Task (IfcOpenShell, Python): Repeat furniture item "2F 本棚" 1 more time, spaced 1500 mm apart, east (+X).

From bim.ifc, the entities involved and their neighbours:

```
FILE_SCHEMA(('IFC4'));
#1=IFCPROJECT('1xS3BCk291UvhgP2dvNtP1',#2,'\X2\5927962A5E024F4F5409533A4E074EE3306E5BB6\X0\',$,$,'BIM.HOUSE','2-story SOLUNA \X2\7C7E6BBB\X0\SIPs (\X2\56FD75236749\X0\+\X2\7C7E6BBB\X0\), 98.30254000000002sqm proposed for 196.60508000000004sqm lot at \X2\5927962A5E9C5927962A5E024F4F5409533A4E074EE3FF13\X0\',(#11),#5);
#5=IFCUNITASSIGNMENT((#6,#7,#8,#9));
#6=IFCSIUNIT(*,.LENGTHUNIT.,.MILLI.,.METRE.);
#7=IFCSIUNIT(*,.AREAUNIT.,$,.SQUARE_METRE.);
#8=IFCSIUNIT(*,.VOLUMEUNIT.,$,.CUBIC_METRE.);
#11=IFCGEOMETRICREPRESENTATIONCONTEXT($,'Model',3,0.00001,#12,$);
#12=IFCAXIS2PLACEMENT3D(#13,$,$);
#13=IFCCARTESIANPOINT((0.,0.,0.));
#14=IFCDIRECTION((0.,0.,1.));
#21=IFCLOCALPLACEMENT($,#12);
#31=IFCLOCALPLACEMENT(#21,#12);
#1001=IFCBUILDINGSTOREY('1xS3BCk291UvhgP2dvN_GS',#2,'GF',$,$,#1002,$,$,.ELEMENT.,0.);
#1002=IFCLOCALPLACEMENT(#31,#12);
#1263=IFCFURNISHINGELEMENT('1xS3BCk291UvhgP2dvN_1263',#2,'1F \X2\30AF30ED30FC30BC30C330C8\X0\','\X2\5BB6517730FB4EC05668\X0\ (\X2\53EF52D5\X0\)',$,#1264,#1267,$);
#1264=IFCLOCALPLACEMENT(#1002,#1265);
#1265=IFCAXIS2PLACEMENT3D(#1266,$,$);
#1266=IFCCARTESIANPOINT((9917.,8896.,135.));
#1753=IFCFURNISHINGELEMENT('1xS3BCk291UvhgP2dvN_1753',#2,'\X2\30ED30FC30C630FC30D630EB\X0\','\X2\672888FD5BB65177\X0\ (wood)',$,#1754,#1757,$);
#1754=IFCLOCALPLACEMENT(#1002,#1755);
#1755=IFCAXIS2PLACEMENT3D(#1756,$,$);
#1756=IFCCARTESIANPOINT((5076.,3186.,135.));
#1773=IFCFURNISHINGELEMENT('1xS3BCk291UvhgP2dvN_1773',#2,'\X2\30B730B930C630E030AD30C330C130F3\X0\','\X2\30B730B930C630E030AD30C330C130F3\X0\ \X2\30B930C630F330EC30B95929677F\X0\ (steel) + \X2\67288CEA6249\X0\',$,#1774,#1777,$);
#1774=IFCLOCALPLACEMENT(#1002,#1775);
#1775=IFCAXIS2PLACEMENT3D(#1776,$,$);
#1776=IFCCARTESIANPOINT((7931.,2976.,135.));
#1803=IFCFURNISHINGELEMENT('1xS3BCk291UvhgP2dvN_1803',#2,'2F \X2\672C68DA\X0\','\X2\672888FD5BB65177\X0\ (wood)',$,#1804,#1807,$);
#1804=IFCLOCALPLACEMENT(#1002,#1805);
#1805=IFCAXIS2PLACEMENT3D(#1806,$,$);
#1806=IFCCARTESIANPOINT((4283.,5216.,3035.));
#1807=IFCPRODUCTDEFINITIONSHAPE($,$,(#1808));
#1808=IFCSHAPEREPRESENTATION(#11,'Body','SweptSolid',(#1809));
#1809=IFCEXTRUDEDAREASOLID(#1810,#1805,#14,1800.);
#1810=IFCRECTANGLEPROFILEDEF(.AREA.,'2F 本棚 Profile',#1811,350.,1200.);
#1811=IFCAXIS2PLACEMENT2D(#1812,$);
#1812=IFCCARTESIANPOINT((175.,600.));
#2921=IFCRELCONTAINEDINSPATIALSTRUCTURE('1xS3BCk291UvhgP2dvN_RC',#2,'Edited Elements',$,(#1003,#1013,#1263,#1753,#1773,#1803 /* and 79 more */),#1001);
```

```python
import numpy as np
import ifcopenshell
import ifcopenshell.api.geometry
import ifcopenshell.api.root
import ifcopenshell.util.element
import ifcopenshell.util.placement

model = ifcopenshell.open("bim.ifc")


def reuse_history(source, copy):
    """copy_class also copies each property set's owner history, people and application; keep the originals."""
    for rel in copy.IsDefinedBy:
        if rel.is_a("IfcRelDefinesByProperties") and (history := rel.RelatingPropertyDefinition.OwnerHistory):
            rel.RelatingPropertyDefinition.OwnerHistory = source.OwnerHistory
            ifcopenshell.util.element.remove_deep2(model, history)


source = model.by_guid("1xS3BCk291UvhgP2dvN_1803")
base = ifcopenshell.util.placement.get_local_placement(source.ObjectPlacement)
step = np.array([1.0, 0.0, 0.0]) * 1500.0

for i in range(1, 2):
    copy = ifcopenshell.api.root.copy_class(model, product=source)
    copy.Representation = ifcopenshell.util.element.copy_deep(
        model, source.Representation, exclude=["IfcGeometricRepresentationContext", "IfcRepresentationMap"]
    )
    reuse_history(source, copy)
    matrix = base.copy()
    matrix[:3, 3] += i * step
    print("added at", matrix[:3, 3].round(3) + 0.0)
    ifcopenshell.api.geometry.edit_object_placement(model, product=copy, matrix=matrix, is_si=False)

model.write("bim-out.ifc")
```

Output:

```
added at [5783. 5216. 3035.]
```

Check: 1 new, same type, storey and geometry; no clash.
